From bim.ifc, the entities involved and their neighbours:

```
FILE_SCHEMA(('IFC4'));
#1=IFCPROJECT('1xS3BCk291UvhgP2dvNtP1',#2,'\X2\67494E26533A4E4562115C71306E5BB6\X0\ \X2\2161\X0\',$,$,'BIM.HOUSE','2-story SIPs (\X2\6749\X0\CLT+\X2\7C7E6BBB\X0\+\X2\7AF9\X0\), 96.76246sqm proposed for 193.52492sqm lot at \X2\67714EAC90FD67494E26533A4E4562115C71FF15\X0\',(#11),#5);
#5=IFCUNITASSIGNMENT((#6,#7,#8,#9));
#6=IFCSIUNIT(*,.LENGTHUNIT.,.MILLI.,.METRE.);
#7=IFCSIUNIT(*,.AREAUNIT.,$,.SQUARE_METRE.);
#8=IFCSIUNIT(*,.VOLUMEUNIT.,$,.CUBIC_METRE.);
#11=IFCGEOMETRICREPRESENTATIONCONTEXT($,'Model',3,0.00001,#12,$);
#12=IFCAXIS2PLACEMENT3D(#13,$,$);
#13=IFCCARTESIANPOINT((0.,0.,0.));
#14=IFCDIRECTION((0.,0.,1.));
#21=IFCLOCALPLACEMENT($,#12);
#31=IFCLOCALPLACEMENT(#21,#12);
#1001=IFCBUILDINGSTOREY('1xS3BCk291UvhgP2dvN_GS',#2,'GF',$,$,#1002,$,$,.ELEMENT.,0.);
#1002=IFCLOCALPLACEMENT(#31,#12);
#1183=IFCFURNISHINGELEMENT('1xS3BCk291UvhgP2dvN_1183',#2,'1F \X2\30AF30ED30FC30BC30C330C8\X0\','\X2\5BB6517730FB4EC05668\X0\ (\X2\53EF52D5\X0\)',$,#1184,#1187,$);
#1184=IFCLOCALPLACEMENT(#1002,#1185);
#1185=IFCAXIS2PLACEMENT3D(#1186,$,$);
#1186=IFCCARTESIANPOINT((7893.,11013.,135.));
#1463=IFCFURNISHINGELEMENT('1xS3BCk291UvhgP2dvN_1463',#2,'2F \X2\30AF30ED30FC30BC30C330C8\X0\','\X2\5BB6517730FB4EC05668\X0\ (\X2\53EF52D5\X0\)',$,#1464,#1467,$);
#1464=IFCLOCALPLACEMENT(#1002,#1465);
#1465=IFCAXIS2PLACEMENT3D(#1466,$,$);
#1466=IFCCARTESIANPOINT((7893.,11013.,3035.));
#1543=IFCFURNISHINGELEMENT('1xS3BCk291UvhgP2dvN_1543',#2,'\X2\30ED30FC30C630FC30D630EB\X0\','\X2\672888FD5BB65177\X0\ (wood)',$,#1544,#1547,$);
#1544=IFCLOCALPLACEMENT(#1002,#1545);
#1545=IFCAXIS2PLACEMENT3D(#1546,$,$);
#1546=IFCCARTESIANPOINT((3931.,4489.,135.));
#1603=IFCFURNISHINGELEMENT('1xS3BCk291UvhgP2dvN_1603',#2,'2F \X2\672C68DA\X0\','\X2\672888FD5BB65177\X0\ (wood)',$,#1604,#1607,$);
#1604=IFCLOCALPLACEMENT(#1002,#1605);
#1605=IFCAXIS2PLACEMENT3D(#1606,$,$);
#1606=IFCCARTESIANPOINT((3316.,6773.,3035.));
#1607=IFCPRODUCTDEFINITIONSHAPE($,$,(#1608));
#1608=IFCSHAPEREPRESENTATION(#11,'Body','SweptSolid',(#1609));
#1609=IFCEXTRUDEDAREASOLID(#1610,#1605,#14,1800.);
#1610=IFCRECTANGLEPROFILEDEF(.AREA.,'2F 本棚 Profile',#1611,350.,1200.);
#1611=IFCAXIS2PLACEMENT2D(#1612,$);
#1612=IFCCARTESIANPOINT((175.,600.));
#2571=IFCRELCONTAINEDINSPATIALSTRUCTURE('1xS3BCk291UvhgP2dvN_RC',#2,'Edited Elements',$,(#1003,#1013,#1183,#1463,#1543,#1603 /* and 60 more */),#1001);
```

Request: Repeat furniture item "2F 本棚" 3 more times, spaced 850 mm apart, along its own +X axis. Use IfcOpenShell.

```python
import ifcopenshell
import ifcopenshell.api.geometry
import ifcopenshell.api.root
import ifcopenshell.util.element
import ifcopenshell.util.placement

model = ifcopenshell.open("bim.ifc")


def reuse_history(source, copy):
    """copy_class also copies each property set's owner history, people and application; keep the originals."""
    for rel in copy.IsDefinedBy:
        if rel.is_a("IfcRelDefinesByProperties") and (history := rel.RelatingPropertyDefinition.OwnerHistory):
            rel.RelatingPropertyDefinition.OwnerHistory = source.OwnerHistory
            ifcopenshell.util.element.remove_deep2(model, history)


source = model.by_guid("1xS3BCk291UvhgP2dvN_1603")
base = ifcopenshell.util.placement.get_local_placement(source.ObjectPlacement)
step = base[:3, 0] * 850.0

for i in range(1, 4):
    copy = ifcopenshell.api.root.copy_class(model, product=source)
    copy.Representation = ifcopenshell.util.element.copy_deep(
        model, source.Representation, exclude=["IfcGeometricRepresentationContext", "IfcRepresentationMap"]
    )
    reuse_history(source, copy)
    matrix = base.copy()
    matrix[:3, 3] += i * step
    print("added at", matrix[:3, 3].round(3) + 0.0)
    ifcopenshell.api.geometry.edit_object_placement(model, product=copy, matrix=matrix, is_si=False)

model.write("bim_updated.ifc")
```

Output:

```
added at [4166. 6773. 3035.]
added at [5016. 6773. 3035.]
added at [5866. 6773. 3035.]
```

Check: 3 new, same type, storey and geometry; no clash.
